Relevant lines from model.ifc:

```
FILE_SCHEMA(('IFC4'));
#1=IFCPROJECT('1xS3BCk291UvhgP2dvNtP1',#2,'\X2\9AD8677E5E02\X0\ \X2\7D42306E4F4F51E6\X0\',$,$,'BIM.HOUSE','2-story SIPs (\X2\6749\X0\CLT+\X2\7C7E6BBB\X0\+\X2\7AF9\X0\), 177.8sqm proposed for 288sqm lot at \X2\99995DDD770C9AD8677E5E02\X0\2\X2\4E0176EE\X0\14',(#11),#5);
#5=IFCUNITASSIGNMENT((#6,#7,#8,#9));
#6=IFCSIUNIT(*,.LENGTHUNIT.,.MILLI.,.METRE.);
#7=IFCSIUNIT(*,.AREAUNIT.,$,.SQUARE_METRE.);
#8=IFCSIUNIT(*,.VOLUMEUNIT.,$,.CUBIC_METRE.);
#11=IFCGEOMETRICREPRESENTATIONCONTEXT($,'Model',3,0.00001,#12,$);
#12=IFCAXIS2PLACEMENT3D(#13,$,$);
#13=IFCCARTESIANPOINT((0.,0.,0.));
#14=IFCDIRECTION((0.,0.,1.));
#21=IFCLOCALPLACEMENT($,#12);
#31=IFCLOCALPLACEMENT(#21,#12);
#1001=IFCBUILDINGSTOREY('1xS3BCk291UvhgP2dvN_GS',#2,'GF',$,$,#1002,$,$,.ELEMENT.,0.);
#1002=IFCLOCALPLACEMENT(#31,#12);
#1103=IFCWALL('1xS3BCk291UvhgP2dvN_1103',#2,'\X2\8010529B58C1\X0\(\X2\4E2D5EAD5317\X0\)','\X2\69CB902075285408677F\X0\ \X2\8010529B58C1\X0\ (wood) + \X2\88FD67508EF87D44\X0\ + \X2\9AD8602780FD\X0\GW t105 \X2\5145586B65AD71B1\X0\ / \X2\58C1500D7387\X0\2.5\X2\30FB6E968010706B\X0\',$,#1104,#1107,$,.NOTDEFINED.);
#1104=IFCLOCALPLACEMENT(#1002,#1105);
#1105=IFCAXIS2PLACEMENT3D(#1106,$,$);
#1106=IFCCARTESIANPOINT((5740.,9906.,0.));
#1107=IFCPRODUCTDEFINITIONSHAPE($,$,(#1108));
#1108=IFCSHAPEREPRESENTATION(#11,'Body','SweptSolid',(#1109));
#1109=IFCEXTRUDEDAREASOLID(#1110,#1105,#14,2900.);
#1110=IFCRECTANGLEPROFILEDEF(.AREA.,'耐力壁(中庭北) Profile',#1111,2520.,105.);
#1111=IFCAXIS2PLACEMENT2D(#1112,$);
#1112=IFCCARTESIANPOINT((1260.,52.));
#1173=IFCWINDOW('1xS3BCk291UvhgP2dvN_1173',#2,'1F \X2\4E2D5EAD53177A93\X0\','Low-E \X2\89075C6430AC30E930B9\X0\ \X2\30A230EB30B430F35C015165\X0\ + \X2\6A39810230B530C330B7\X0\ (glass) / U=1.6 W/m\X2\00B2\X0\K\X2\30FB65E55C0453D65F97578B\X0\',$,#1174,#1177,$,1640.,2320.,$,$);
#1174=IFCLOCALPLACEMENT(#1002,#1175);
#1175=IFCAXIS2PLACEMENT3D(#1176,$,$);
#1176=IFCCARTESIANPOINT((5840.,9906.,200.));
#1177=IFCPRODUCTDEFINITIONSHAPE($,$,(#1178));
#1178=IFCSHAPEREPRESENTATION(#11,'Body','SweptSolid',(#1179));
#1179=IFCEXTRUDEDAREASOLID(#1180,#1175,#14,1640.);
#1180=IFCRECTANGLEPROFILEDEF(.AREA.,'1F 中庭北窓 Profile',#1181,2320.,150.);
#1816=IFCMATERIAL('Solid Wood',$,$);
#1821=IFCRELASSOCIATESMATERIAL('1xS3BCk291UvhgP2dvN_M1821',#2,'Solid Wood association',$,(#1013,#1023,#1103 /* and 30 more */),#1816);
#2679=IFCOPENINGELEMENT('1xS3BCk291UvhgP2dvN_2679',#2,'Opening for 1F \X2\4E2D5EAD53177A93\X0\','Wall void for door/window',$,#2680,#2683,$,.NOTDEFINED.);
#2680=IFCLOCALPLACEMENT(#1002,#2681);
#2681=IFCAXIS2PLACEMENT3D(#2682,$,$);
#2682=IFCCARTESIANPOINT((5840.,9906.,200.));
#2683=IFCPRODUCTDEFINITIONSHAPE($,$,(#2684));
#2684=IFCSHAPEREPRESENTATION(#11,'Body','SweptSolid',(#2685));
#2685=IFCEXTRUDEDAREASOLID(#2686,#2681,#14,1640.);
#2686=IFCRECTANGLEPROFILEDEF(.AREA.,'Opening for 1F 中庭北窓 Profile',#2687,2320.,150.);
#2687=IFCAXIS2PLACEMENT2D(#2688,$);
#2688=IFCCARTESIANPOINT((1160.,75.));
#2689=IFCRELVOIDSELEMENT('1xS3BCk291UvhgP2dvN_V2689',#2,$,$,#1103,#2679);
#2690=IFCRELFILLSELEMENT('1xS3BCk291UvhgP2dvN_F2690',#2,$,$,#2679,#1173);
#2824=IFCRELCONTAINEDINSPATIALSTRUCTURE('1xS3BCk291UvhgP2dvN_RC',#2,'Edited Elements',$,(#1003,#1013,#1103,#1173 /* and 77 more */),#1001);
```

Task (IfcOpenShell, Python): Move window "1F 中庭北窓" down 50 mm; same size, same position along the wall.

```python
import numpy as np
import ifcopenshell
import ifcopenshell.api.geometry
import ifcopenshell.util.placement
import ifcopenshell.util.unit

model = ifcopenshell.open("model.ifc")
unit_scale = ifcopenshell.util.unit.calculate_unit_scale(model)

window = model.by_id(1173)
opening = window.FillsVoids[0].RelatingOpeningElement
dz = -50.0

shift = np.array([0.0, 0.0, dz])
# The window is not placed relative to its opening, so move both.
for product in (opening, window):
    matrix = ifcopenshell.util.placement.get_local_placement(product.ObjectPlacement)
    matrix[:3, 3] += shift
    ifcopenshell.api.geometry.edit_object_placement(model, product=product, matrix=matrix, is_si=False)

print(f"moved by {dz * unit_scale:+.3f} m")

model.write("model_edited.ifc")
```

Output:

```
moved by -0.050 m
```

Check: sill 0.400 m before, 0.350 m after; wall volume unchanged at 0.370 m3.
